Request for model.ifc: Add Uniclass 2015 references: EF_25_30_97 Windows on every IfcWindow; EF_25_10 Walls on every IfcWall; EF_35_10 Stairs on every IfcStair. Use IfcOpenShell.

First a look at what the model holds.

```python
import ifcopenshell

model = ifcopenshell.open("model.ifc")
print(model.schema)
print("classifications:", [c.Name for c in model.by_type("IfcClassification")])
for ifc_class in ("IfcDoor", "IfcRoof", "IfcStair", "IfcWall", "IfcWindow"):
    print(ifc_class, len(model.by_type(ifc_class)))
```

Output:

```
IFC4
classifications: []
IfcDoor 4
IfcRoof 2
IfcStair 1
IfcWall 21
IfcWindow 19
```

```python
import ifcopenshell
import ifcopenshell.api.classification

model = ifcopenshell.open("model.ifc")

system = ifcopenshell.api.classification.add_classification(model, classification="Uniclass 2015")

codes = {
    "IfcWindow": ("EF_25_30_97", "Windows"),
    "IfcWall": ("EF_25_10", "Walls"),
    "IfcStair": ("EF_35_10", "Stairs"),
}
for ifc_class, (code, name) in codes.items():
    products = model.by_type(ifc_class)
    ifcopenshell.api.classification.add_reference(
        model, products=products, classification=system, identification=code, name=name
    )
    print(code, len(products))

model.write("model_v2.ifc")
```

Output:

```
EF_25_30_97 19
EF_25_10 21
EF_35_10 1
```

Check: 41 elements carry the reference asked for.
